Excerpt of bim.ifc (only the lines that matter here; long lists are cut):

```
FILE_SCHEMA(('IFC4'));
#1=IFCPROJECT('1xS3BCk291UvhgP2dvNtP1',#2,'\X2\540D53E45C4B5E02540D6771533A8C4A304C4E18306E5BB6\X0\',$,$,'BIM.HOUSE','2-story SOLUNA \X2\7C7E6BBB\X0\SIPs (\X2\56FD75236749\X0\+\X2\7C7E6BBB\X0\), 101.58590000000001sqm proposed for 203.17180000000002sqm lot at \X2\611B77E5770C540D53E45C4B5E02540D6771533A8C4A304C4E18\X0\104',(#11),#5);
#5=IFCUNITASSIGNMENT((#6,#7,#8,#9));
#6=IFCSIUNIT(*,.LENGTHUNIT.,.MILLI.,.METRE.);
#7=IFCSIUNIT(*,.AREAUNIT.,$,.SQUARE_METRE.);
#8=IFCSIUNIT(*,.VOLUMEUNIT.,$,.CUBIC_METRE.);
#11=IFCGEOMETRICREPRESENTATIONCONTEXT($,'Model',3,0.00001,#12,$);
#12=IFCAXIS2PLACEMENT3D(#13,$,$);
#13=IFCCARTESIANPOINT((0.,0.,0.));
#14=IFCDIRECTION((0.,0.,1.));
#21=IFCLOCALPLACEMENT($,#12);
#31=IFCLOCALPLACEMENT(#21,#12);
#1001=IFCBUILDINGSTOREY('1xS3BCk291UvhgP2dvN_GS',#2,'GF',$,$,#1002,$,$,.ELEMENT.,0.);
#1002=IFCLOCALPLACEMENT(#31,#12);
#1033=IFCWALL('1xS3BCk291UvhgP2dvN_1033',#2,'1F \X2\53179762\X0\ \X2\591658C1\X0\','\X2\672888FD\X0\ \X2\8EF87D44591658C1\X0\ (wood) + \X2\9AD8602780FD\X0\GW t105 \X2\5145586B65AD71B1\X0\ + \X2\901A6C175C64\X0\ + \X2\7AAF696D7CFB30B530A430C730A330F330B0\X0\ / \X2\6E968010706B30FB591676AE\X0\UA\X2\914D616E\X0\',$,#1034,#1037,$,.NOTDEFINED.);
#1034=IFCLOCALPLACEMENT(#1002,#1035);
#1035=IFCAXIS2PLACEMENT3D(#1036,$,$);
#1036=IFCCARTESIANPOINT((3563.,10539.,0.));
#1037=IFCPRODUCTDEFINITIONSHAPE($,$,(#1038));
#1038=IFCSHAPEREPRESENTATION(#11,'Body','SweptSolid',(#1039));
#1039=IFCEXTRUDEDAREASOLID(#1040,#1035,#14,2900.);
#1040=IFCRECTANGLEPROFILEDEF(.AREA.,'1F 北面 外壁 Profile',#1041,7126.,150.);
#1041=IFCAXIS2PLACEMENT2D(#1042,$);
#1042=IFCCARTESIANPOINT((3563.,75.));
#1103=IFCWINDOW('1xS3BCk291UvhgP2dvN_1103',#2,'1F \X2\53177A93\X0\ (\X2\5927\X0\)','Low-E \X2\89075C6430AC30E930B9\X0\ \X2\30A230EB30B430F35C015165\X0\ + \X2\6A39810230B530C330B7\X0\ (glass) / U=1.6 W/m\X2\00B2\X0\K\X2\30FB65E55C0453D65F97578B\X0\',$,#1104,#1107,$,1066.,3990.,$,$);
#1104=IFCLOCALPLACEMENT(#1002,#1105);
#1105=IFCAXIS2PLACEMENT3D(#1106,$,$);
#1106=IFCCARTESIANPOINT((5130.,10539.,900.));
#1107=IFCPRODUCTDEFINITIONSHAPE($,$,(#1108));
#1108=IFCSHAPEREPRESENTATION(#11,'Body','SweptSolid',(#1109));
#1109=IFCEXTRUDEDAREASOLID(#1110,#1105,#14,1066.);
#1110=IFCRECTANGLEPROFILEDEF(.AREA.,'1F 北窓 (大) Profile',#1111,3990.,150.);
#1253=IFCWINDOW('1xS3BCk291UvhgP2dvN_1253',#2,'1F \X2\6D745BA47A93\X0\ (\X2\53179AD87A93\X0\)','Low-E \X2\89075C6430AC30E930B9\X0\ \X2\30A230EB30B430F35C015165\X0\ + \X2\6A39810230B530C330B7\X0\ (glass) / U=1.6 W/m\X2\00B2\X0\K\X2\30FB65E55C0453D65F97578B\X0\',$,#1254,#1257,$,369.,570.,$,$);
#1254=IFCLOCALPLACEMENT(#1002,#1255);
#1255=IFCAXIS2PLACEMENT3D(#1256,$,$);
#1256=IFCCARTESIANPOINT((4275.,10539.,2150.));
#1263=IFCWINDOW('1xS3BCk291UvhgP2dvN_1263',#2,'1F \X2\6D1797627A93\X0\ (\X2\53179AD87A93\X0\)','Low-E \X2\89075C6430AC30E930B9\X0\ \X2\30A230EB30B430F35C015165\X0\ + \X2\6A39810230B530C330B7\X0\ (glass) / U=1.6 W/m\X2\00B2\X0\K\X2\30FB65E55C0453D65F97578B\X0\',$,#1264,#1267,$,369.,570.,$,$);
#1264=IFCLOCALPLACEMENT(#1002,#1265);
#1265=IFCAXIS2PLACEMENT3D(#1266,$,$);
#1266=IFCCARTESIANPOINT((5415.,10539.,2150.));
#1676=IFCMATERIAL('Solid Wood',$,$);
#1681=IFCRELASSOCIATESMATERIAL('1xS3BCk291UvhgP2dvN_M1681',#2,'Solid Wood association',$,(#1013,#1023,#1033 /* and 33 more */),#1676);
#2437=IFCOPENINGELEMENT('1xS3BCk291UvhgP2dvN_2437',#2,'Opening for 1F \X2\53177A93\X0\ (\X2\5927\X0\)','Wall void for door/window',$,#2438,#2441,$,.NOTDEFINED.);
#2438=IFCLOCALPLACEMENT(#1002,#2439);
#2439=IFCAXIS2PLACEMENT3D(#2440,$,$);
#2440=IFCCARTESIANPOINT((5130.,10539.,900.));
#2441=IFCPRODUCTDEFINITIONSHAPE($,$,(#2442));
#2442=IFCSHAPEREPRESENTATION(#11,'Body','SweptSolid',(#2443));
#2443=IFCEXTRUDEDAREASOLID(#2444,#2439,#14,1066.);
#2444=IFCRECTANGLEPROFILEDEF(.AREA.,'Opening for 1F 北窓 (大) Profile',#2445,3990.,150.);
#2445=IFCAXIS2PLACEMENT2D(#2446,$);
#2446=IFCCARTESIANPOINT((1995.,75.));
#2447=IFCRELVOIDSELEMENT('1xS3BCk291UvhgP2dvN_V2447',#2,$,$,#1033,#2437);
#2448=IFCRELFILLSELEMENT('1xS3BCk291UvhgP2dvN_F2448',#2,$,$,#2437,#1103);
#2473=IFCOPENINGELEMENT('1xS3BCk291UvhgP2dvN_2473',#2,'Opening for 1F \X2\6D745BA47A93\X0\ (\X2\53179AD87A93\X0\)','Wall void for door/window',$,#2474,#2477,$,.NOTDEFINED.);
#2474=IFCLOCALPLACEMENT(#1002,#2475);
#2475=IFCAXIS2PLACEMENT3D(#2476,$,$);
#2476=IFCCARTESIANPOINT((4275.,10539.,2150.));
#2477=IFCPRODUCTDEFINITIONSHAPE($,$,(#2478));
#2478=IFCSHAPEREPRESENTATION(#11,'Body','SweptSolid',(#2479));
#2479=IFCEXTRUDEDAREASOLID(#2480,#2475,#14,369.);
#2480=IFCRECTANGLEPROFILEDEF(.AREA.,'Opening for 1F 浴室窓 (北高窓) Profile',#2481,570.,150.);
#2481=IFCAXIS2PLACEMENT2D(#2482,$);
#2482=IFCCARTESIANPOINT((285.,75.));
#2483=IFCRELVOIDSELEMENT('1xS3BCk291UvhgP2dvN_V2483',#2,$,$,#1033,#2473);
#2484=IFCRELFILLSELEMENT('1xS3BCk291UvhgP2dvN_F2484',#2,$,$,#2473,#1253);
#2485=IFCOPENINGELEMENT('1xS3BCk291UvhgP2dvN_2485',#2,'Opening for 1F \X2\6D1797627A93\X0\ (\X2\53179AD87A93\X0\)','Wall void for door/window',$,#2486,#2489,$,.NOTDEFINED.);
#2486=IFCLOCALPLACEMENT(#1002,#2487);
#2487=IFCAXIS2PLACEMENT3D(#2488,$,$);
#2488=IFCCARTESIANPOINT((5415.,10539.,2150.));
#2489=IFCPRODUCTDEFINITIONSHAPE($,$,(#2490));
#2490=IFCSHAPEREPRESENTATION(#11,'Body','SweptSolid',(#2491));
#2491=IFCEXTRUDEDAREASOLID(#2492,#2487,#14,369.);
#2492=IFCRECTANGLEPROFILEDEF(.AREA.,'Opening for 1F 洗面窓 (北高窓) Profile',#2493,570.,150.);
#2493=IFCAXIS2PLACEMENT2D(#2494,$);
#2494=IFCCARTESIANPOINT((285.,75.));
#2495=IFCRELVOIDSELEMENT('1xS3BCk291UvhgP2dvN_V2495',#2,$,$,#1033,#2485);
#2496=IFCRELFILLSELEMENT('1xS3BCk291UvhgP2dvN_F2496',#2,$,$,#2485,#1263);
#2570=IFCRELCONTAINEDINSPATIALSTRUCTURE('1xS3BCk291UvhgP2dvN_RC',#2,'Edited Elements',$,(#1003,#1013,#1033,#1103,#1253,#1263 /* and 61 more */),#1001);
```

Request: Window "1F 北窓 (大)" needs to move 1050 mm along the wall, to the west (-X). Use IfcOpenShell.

```python
import ifcopenshell
import ifcopenshell.api.geometry
import ifcopenshell.util.placement
import ifcopenshell.util.unit

model = ifcopenshell.open("bim.ifc")
unit_scale = ifcopenshell.util.unit.calculate_unit_scale(model)

window = model.by_guid("1xS3BCk291UvhgP2dvN_1103")
opening = window.FillsVoids[0].RelatingOpeningElement
wall = opening.VoidsElements[0].RelatingBuildingElement

wall_matrix = ifcopenshell.util.placement.get_local_placement(wall.ObjectPlacement)
shift = wall_matrix[:3, 0] * -1.05 / unit_scale
before = ifcopenshell.util.placement.get_local_placement(window.ObjectPlacement)[:3, 3].copy()

# The window is not placed relative to its opening, so move both.
for product in (opening, window):
    matrix = ifcopenshell.util.placement.get_local_placement(product.ObjectPlacement)
    matrix[:3, 3] += shift
    ifcopenshell.api.geometry.edit_object_placement(model, product=product, matrix=matrix, is_si=False)

after = ifcopenshell.util.placement.get_local_placement(window.ObjectPlacement)[:3, 3]
print("window moved by", (after - before).round(3) + 0.0)

model.write("bim_rev.ifc")
```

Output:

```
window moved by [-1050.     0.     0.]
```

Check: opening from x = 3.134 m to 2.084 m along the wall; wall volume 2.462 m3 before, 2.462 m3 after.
